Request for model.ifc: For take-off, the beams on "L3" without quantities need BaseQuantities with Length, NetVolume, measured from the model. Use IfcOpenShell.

First a look at what the model holds.

```python
import ifcopenshell
import ifcopenshell.util.element
import ifcopenshell.util.unit

model = ifcopenshell.open("model.ifc")
print(model.schema)
for unit_type in ("LENGTHUNIT", "AREAUNIT", "VOLUMEUNIT"):
    print(unit_type, ifcopenshell.util.unit.calculate_unit_scale(model, unit_type))
storey = next(s for s in model.by_type("IfcBuildingStorey") if s.Name == "L3")
beams = [e for e in ifcopenshell.util.element.get_decomposition(storey) if e.is_a("IfcBeam")]
for e in sorted(beams, key=lambda e: e.id()):
    print(e.id(), e.is_a(), e.Name, list(ifcopenshell.util.element.get_psets(e, qtos_only=True)), sep=" | ")
```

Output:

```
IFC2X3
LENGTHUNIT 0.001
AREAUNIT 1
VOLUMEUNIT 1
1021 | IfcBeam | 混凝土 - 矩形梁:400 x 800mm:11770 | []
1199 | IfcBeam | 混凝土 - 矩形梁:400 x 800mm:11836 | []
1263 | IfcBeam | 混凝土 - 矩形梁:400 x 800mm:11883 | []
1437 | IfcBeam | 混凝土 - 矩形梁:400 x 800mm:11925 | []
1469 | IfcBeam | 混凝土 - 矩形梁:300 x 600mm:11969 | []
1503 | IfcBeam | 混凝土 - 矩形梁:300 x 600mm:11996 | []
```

```python
import ifcopenshell
import ifcopenshell.api.pset
import ifcopenshell.geom
import ifcopenshell.util.element
import ifcopenshell.util.shape
import ifcopenshell.util.unit

model = ifcopenshell.open("model.ifc")
unit_scale = ifcopenshell.util.unit.calculate_unit_scale(model)
volume_scale = ifcopenshell.util.unit.calculate_unit_scale(model, "VOLUMEUNIT")
settings = ifcopenshell.geom.settings()

storey = next(s for s in model.by_type("IfcBuildingStorey") if s.Name == "L3")
beams = [e for e in ifcopenshell.util.element.get_decomposition(storey) if e.is_a("IfcBeam")]

for e in sorted(beams, key=lambda e: e.id()):
    if ifcopenshell.util.element.get_psets(e, qtos_only=True, should_inherit=False):
        continue
    # Geometry comes back in metres, in the element's own axes.
    shape = ifcopenshell.geom.create_shape(settings, e)
    values = {
        "Length": ifcopenshell.util.shape.get_max_xyz(shape.geometry) / unit_scale,
        "NetVolume": ifcopenshell.util.shape.get_volume(shape.geometry) / volume_scale,
    }
    qto = ifcopenshell.api.pset.add_qto(model, product=e, name="BaseQuantities")
    ifcopenshell.api.pset.edit_qto(model, qto=qto, properties=values)
    print(e.id(), {k: round(v, 3) for k, v in values.items()})

model.write("model_rev.ifc")
```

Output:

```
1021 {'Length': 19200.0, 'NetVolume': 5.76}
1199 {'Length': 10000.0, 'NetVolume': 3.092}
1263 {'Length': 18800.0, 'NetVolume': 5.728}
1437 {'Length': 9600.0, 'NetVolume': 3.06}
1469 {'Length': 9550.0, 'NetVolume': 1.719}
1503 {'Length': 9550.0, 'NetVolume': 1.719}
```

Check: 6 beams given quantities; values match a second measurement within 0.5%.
